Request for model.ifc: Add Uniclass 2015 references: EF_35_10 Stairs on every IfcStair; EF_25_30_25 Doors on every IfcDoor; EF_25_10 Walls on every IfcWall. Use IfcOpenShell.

First a look at what the model holds.

```python
import ifcopenshell

model = ifcopenshell.open("model.ifc")
print(model.schema)
print("classifications:", [c.Name for c in model.by_type("IfcClassification")])
for ifc_class in ("IfcDoor", "IfcRoof", "IfcStair", "IfcWall", "IfcWindow"):
    print(ifc_class, len(model.by_type(ifc_class)))
```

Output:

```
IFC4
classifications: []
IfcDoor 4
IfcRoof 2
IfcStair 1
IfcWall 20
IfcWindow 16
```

```python
import ifcopenshell
import ifcopenshell.api.classification

model = ifcopenshell.open("model.ifc")

system = ifcopenshell.api.classification.add_classification(model, classification="Uniclass 2015")

codes = {
    "IfcStair": ("EF_35_10", "Stairs"),
    "IfcDoor": ("EF_25_30_25", "Doors"),
    "IfcWall": ("EF_25_10", "Walls"),
}
for ifc_class, (code, name) in codes.items():
    products = model.by_type(ifc_class)
    ifcopenshell.api.classification.add_reference(
        model, products=products, classification=system, identification=code, name=name
    )
    print(code, len(products))

model.write("model-out.ifc")
```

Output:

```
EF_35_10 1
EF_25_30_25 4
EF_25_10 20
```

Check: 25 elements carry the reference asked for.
